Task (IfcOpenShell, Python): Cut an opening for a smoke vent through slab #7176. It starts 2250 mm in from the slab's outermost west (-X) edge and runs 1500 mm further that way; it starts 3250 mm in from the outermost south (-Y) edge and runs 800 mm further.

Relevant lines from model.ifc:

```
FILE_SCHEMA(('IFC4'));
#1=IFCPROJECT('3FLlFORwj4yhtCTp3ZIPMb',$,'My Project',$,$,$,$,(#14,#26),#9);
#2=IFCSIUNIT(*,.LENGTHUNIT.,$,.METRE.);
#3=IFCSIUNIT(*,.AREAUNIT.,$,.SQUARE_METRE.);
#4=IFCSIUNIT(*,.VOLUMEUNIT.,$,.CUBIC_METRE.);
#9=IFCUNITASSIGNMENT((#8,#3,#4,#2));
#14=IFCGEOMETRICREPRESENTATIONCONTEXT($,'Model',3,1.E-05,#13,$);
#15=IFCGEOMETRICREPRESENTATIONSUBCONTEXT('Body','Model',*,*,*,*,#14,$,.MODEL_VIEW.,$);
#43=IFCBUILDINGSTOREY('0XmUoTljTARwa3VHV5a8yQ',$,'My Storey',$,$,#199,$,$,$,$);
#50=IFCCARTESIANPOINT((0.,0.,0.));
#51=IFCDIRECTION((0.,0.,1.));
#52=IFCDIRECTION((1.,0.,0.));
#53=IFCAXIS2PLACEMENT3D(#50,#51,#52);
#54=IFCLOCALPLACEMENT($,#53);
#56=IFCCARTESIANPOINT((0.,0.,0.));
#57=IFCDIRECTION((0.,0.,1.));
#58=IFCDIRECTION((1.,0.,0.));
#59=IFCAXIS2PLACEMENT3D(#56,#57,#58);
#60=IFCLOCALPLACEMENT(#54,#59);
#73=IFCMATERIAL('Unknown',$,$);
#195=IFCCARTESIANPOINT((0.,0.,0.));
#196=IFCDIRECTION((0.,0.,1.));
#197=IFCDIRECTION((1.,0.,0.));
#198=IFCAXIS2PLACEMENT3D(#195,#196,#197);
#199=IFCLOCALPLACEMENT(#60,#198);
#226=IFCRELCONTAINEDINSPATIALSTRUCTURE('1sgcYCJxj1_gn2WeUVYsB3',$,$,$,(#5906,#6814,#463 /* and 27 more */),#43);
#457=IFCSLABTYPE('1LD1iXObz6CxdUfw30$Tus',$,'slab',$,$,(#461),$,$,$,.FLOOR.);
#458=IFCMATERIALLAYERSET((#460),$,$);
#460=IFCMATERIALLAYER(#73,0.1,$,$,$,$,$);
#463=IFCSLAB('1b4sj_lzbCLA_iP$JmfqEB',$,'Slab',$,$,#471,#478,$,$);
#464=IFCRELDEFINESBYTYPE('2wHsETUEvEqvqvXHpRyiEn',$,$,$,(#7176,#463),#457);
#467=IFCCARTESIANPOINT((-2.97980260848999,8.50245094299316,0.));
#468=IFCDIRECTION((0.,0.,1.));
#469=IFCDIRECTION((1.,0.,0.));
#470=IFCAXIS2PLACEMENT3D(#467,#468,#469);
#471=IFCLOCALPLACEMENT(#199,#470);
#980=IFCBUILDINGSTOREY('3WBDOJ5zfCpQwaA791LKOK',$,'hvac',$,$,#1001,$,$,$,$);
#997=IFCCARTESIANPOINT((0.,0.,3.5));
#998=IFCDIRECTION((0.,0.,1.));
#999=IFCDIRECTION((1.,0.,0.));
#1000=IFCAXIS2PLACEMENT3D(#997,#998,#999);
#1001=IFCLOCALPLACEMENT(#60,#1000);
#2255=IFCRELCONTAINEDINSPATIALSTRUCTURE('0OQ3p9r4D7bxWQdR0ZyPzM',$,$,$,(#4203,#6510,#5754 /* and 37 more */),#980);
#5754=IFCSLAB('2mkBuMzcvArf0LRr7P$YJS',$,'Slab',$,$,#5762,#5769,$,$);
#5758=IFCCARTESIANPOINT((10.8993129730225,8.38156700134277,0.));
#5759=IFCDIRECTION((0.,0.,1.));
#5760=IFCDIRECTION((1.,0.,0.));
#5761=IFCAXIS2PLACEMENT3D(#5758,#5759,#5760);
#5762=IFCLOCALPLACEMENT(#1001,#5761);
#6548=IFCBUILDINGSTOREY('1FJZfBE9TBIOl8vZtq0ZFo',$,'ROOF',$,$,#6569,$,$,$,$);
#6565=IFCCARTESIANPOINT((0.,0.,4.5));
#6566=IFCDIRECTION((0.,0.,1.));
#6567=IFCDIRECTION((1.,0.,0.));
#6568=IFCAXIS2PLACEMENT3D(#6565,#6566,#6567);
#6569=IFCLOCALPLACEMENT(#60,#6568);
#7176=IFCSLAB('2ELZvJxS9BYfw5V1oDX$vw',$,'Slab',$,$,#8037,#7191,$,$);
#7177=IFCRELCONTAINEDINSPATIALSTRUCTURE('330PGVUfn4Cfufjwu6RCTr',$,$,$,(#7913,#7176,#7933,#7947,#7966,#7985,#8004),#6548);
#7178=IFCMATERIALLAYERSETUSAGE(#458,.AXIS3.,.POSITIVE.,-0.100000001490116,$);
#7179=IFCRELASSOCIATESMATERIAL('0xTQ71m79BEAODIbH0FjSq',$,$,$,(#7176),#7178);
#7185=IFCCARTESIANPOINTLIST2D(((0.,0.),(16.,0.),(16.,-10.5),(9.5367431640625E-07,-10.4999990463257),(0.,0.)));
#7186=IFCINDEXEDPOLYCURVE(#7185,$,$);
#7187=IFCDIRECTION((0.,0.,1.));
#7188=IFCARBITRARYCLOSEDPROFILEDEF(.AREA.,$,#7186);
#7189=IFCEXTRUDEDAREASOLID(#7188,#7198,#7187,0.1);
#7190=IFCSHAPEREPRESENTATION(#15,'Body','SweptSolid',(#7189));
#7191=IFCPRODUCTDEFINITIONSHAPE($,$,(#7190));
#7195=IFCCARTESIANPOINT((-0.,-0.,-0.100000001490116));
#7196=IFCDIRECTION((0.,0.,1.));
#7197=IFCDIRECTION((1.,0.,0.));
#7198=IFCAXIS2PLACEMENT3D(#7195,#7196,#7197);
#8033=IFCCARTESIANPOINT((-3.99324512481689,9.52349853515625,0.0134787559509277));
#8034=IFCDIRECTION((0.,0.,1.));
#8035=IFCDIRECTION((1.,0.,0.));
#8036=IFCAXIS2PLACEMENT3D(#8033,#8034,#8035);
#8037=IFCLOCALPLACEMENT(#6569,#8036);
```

```python
import numpy as np
import ifcopenshell
import ifcopenshell.api.feature
import ifcopenshell.api.geometry
import ifcopenshell.api.root
import ifcopenshell.geom
import ifcopenshell.util.placement
import ifcopenshell.util.representation
import ifcopenshell.util.shape
import ifcopenshell.util.unit

model = ifcopenshell.open("model.ifc")
unit_scale = ifcopenshell.util.unit.calculate_unit_scale(model)
settings = ifcopenshell.geom.settings()


def volume(element):
    """Net volume in cubic metres, openings subtracted."""
    shape = ifcopenshell.geom.create_shape(settings, element)
    return ifcopenshell.util.shape.get_volume(shape.geometry)


slab = model.by_guid("2ELZvJxS9BYfw5V1oDX$vw")
before = volume(slab)

# Extent in the slab's own axes, in metres. The edges named are its -X and -Y sides.
slab_shape = ifcopenshell.geom.create_shape(settings, slab)
vertices = ifcopenshell.util.shape.get_vertices(slab_shape.geometry)
x_min, y_min, bottom = vertices.min(axis=0)
top = vertices[:, 2].max()

opening = ifcopenshell.api.root.create_entity(model, ifc_class="IfcOpeningElement", name="Smoke vent opening", predefined_type="OPENING")
context = ifcopenshell.util.representation.get_context(model, "Model", "Body", "MODEL_VIEW")
width, depth = 1.5, 0.8
outline = [(0.0, 0.0), (width, 0.0), (width, depth), (0.0, depth), (0.0, 0.0)]
# Overshoot both faces by 50 mm so the cut is clean.
shape = ifcopenshell.api.geometry.add_slab_representation(
    model, context=context, depth=top - bottom + 0.1, polyline=outline
)
ifcopenshell.api.geometry.assign_representation(model, product=opening, representation=shape)

matrix = ifcopenshell.util.placement.get_local_placement(slab.ObjectPlacement)
matrix[:, 3] = matrix @ np.append(np.array([x_min + 2.25, y_min + 3.25, bottom - 0.05]) / unit_scale, 1.0)
ifcopenshell.api.geometry.edit_object_placement(model, product=opening, matrix=matrix, is_si=False)
ifcopenshell.api.feature.add_feature(model, feature=opening, element=slab)

after = volume(slab)

print(f"slab volume {before:.3f} -> {after:.3f} m3")

model.write("model_rev.ifc")
```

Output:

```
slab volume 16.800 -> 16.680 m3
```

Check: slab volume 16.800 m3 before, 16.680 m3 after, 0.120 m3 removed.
